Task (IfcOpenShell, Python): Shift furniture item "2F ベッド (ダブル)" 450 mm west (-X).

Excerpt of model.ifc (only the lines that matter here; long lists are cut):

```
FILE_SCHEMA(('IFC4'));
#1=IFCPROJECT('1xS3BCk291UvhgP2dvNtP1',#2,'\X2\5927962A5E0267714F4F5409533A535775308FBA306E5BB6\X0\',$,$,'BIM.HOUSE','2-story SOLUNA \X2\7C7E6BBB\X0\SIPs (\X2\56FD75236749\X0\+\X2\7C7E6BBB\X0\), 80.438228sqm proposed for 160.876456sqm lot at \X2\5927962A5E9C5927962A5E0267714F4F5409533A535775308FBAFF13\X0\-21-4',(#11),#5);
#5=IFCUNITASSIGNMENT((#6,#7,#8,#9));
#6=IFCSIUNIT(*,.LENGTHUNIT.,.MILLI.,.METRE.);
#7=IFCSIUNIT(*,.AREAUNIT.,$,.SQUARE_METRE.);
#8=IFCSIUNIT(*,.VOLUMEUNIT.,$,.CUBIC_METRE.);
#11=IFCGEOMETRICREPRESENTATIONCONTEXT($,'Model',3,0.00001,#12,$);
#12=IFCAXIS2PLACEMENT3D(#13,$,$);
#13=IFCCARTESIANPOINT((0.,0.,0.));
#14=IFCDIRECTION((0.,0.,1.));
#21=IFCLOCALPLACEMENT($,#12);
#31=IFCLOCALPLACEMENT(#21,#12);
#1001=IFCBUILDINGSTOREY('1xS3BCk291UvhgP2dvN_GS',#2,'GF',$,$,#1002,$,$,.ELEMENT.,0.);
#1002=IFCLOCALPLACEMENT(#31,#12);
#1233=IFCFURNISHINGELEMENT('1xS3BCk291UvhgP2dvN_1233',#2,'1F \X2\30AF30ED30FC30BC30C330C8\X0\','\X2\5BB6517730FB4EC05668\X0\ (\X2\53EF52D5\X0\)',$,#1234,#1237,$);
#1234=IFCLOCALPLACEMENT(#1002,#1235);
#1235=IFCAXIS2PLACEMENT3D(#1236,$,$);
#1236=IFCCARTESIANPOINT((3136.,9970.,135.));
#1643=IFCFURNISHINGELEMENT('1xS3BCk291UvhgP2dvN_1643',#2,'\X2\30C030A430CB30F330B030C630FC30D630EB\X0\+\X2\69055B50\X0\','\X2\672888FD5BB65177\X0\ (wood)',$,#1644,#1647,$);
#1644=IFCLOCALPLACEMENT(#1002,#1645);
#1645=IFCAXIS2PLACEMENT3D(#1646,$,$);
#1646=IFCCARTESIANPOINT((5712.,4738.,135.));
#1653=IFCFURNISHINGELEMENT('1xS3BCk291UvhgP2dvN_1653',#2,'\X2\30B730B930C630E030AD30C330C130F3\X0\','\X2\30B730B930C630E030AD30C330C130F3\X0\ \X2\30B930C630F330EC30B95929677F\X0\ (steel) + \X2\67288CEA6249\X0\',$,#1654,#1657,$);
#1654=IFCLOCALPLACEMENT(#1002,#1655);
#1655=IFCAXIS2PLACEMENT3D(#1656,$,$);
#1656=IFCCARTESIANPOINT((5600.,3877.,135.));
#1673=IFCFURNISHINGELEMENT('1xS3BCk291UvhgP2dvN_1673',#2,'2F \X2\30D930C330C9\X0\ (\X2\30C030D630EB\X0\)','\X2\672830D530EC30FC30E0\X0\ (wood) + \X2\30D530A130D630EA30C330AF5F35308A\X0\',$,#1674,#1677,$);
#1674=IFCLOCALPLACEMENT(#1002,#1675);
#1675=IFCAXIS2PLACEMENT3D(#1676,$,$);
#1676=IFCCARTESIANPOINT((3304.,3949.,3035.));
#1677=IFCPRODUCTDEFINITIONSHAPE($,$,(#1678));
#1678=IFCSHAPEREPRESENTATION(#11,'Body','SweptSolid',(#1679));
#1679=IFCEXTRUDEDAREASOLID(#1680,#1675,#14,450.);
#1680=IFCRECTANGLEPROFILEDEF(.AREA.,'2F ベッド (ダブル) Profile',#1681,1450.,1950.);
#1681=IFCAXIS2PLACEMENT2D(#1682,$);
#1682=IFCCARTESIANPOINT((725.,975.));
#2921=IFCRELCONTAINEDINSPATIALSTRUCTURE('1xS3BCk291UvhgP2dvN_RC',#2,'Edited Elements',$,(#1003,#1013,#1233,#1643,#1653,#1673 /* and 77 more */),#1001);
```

```python
import ifcopenshell
import ifcopenshell.api.geometry
import ifcopenshell.util.placement

model = ifcopenshell.open("model.ifc")

item = model.by_guid("1xS3BCk291UvhgP2dvN_1673")
matrix = ifcopenshell.util.placement.get_local_placement(item.ObjectPlacement)
matrix[0, 3] -= 450.0
ifcopenshell.api.geometry.edit_object_placement(model, product=item, matrix=matrix, is_si=False)

print(ifcopenshell.util.placement.get_local_placement(item.ObjectPlacement).round(3) + 0.0)

model.write("model_edited.ifc")
```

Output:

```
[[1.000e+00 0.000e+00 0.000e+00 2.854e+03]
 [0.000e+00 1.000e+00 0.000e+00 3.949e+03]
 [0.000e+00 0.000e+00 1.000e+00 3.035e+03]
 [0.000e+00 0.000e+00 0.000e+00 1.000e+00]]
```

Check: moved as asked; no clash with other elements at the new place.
